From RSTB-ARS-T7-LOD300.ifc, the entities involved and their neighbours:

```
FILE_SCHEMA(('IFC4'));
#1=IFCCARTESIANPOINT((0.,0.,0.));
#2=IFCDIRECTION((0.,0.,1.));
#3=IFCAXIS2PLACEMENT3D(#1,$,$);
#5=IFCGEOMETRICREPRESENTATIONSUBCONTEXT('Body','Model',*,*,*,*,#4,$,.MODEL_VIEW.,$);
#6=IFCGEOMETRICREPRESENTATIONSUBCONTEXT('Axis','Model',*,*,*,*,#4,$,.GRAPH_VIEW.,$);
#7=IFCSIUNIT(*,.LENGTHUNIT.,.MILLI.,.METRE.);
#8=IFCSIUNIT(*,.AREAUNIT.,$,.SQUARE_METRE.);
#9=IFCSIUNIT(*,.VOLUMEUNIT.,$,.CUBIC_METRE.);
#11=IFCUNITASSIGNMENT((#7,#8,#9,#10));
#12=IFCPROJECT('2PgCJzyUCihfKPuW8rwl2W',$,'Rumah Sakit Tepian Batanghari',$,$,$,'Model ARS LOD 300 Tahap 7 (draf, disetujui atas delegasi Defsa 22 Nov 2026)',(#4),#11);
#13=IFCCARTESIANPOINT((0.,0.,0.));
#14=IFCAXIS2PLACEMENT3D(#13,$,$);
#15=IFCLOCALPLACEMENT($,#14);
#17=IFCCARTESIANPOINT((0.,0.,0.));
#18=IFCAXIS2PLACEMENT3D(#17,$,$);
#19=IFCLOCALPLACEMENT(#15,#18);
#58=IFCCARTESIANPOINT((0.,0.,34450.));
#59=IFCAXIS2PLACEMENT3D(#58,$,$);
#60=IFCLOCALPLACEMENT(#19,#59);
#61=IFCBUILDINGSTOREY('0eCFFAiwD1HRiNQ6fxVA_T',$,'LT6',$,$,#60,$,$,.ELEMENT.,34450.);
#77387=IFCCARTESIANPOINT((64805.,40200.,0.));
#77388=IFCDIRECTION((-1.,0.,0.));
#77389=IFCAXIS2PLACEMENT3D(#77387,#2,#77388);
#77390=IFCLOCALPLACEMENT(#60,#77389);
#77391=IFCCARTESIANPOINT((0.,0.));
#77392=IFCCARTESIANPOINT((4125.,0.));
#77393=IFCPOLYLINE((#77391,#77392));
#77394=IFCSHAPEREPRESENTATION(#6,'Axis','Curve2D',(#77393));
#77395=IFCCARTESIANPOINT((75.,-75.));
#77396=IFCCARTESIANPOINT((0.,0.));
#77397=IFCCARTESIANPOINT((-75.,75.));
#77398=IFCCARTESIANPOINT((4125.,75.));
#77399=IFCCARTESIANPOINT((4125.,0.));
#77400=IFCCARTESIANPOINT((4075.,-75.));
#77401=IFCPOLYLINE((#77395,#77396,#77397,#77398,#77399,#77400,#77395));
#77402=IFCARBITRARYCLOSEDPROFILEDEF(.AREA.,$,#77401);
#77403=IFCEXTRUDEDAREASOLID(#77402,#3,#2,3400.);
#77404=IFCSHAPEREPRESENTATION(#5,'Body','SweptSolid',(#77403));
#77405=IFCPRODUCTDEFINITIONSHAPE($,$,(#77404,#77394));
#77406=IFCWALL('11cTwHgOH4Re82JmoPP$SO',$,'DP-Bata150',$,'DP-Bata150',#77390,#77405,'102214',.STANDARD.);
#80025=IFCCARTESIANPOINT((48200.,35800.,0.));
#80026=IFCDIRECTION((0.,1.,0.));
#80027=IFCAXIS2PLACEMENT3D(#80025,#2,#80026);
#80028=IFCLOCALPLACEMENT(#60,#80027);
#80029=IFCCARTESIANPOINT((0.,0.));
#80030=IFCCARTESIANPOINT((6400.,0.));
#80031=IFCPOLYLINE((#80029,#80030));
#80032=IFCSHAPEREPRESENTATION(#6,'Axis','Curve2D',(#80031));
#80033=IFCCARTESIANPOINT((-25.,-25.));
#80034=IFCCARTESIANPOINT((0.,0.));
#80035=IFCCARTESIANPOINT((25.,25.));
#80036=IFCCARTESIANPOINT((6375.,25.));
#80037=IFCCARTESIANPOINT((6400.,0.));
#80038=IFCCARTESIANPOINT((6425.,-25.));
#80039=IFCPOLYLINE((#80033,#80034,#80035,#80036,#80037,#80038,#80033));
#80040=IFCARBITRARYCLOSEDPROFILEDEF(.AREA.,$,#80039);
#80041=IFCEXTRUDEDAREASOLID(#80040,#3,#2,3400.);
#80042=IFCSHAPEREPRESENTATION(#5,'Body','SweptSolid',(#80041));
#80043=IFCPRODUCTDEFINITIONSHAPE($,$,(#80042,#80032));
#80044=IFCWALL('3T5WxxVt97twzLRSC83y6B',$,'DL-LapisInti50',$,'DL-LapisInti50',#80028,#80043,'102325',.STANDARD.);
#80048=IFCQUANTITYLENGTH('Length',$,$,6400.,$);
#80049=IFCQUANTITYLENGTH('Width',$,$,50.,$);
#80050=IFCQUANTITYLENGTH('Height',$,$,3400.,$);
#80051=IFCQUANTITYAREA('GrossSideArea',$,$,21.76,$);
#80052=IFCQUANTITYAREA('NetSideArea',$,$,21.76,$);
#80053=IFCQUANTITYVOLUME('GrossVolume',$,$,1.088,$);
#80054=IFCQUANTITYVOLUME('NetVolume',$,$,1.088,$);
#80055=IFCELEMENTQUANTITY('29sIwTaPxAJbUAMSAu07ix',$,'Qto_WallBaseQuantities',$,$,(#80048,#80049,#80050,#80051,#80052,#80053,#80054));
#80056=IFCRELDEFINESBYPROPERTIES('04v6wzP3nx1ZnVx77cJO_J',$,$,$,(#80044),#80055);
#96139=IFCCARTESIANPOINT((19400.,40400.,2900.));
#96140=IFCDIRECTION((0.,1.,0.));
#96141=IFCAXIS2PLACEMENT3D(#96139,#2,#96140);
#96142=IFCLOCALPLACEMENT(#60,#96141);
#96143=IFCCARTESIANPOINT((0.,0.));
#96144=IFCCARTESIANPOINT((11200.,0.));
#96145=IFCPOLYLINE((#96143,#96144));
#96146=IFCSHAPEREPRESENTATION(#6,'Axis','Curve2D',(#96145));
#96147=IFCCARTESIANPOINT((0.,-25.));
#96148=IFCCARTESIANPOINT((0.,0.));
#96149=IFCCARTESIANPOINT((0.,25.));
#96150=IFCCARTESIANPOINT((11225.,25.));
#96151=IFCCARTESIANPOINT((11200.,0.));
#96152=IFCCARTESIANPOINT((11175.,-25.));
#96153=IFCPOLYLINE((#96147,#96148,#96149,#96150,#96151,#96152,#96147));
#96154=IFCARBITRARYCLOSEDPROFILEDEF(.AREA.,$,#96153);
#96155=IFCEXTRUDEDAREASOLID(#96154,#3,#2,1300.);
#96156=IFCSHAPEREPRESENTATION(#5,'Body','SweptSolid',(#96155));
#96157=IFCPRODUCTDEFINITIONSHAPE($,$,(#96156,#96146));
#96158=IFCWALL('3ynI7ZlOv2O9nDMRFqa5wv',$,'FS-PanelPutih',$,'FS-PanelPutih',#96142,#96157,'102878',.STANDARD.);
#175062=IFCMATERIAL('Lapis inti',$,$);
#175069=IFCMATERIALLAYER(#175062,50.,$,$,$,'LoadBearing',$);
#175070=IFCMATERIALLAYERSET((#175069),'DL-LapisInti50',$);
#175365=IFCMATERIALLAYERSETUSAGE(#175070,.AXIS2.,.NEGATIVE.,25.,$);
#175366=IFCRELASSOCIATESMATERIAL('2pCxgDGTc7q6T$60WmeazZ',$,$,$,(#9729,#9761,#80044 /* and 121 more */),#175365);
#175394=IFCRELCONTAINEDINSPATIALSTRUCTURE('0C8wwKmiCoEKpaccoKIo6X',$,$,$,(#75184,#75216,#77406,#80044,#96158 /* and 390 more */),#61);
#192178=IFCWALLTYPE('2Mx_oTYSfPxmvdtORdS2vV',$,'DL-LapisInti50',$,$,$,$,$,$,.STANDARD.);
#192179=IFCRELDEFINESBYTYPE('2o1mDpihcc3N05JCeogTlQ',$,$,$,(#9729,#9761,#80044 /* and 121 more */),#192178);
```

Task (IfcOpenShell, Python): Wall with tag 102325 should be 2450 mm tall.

```python
import ifcopenshell
import ifcopenshell.api.pset
import ifcopenshell.geom
import ifcopenshell.util.element
import ifcopenshell.util.representation
import ifcopenshell.util.shape
import ifcopenshell.util.unit

model = ifcopenshell.open("RSTB-ARS-T7-LOD300.ifc")
unit_scale = ifcopenshell.util.unit.calculate_unit_scale(model)
area_scale = ifcopenshell.util.unit.calculate_unit_scale(model, "AREAUNIT")
volume_scale = ifcopenshell.util.unit.calculate_unit_scale(model, "VOLUMEUNIT")
settings = ifcopenshell.geom.settings()


def volume(element):
    """Net volume in cubic metres, openings subtracted."""
    shape = ifcopenshell.geom.create_shape(settings, element)
    return ifcopenshell.util.shape.get_volume(shape.geometry)


wall = model.by_id(80044)
before = volume(wall)

body = ifcopenshell.util.representation.get_representation(wall, "Model", "Body")
solid = body.Items[0]
old_height = solid.Depth
solid.Depth = 2.45 / unit_scale
after = volume(wall)
thickness = 0.05  # wall thickness in metres

# Update the stored height, areas and volumes.
qto = model.by_id(ifcopenshell.util.element.get_pset(wall, "Qto_WallBaseQuantities", should_inherit=False)["id"])
ifcopenshell.api.pset.edit_qto(model, qto=qto, properties={
    "Height": solid.Depth,
    "GrossSideArea": ifcopenshell.util.element.get_pset(wall, "Qto_WallBaseQuantities", "GrossSideArea") * solid.Depth / old_height,
    "NetSideArea": after / thickness / area_scale,
    "GrossVolume": ifcopenshell.util.element.get_pset(wall, "Qto_WallBaseQuantities", "GrossVolume") * solid.Depth / old_height,
    "NetVolume": after / volume_scale,
})

print(f"height {old_height:g} -> {solid.Depth:g}, volume {before:.3f} -> {after:.3f} m3")

model.write("RSTB-ARS-T7-LOD300-out.ifc")
```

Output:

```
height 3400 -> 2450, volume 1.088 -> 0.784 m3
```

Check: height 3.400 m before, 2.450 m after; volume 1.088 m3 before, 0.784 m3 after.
